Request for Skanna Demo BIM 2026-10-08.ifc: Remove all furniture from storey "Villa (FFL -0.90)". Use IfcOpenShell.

First a look at what the model holds.

```python
import ifcopenshell
import ifcopenshell.util.element

model = ifcopenshell.open("Skanna Demo BIM 2026-10-08.ifc")
print(model.schema)
storey = next(s for s in model.by_type("IfcBuildingStorey") if s.Name == "Villa (FFL -0.90)")
furniture = [e for e in ifcopenshell.util.element.get_decomposition(storey) if e.is_a("IfcFurnishingElement")]
seen = {}
for e in furniture:
    element_type = ifcopenshell.util.element.get_type(e)
    name = element_type.Name if element_type not in (None, e) else None
    seen[name] = seen.get(name, 0) + 1
for name, count in sorted(seen.items(), key=str):
    print(count, "x", name)
```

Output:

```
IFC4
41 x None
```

```python
import ifcopenshell
import ifcopenshell.api.root
import ifcopenshell.util.element

model = ifcopenshell.open("Skanna Demo BIM 2026-10-08.ifc")

storey = next(s for s in model.by_type("IfcBuildingStorey") if s.Name == "Villa (FFL -0.90)")
furniture = [e for e in ifcopenshell.util.element.get_decomposition(storey) if e.is_a("IfcFurnishingElement")]

for e in furniture:
    ifcopenshell.api.root.remove_product(model, product=e)
print(len(furniture), "removed")

model.write("Skanna Demo BIM 2026-10-08_edited.ifc")
```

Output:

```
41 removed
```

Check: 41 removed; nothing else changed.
